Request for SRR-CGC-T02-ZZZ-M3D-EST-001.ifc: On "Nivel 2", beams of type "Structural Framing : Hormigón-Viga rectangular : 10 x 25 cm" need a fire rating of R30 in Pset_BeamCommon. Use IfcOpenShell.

First a look at what the model holds.

```python
import ifcopenshell
import ifcopenshell.util.element

model = ifcopenshell.open("SRR-CGC-T02-ZZZ-M3D-EST-001.ifc")
print(model.schema)
storey = next(s for s in model.by_type("IfcBuildingStorey") if s.Name == "Nivel 2")
beams = [e for e in ifcopenshell.util.element.get_decomposition(storey) if e.is_a("IfcBeam")]
seen = {}
for e in beams:
    element_type = ifcopenshell.util.element.get_type(e)
    key = (element_type.Name if element_type != e and element_type else None, ifcopenshell.util.element.get_pset(e, "Pset_BeamCommon", "FireRating"))
    seen[key] = seen.get(key, 0) + 1
for (name, value), count in sorted(seen.items(), key=str):
    print(count, "x", name, "|", value)
```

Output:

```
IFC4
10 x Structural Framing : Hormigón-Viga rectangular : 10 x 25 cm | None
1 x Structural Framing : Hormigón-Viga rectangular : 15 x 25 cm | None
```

```python
import ifcopenshell
import ifcopenshell.api.pset
import ifcopenshell.util.element

model = ifcopenshell.open("SRR-CGC-T02-ZZZ-M3D-EST-001.ifc")

storey = next(s for s in model.by_type("IfcBuildingStorey") if s.Name == "Nivel 2")
beams = [e for e in ifcopenshell.util.element.get_decomposition(storey) if e.is_a("IfcBeam")]

count = 0
for e in beams:
    element_type = ifcopenshell.util.element.get_type(e)
    if element_type in (None, e) or element_type.Name != "Structural Framing : Hormigón-Viga rectangular : 10 x 25 cm":
        continue
    # add_pset returns the element's existing set when there is one.
    pset = ifcopenshell.api.pset.add_pset(model, product=e, name="Pset_BeamCommon")
    ifcopenshell.api.pset.edit_pset(model, pset=pset, properties={"FireRating": "R30"})
    count += 1

print(count, "beams updated")

model.write("SRR-CGC-T02-ZZZ-M3D-EST-001-out.ifc")
```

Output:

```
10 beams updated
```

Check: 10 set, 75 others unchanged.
